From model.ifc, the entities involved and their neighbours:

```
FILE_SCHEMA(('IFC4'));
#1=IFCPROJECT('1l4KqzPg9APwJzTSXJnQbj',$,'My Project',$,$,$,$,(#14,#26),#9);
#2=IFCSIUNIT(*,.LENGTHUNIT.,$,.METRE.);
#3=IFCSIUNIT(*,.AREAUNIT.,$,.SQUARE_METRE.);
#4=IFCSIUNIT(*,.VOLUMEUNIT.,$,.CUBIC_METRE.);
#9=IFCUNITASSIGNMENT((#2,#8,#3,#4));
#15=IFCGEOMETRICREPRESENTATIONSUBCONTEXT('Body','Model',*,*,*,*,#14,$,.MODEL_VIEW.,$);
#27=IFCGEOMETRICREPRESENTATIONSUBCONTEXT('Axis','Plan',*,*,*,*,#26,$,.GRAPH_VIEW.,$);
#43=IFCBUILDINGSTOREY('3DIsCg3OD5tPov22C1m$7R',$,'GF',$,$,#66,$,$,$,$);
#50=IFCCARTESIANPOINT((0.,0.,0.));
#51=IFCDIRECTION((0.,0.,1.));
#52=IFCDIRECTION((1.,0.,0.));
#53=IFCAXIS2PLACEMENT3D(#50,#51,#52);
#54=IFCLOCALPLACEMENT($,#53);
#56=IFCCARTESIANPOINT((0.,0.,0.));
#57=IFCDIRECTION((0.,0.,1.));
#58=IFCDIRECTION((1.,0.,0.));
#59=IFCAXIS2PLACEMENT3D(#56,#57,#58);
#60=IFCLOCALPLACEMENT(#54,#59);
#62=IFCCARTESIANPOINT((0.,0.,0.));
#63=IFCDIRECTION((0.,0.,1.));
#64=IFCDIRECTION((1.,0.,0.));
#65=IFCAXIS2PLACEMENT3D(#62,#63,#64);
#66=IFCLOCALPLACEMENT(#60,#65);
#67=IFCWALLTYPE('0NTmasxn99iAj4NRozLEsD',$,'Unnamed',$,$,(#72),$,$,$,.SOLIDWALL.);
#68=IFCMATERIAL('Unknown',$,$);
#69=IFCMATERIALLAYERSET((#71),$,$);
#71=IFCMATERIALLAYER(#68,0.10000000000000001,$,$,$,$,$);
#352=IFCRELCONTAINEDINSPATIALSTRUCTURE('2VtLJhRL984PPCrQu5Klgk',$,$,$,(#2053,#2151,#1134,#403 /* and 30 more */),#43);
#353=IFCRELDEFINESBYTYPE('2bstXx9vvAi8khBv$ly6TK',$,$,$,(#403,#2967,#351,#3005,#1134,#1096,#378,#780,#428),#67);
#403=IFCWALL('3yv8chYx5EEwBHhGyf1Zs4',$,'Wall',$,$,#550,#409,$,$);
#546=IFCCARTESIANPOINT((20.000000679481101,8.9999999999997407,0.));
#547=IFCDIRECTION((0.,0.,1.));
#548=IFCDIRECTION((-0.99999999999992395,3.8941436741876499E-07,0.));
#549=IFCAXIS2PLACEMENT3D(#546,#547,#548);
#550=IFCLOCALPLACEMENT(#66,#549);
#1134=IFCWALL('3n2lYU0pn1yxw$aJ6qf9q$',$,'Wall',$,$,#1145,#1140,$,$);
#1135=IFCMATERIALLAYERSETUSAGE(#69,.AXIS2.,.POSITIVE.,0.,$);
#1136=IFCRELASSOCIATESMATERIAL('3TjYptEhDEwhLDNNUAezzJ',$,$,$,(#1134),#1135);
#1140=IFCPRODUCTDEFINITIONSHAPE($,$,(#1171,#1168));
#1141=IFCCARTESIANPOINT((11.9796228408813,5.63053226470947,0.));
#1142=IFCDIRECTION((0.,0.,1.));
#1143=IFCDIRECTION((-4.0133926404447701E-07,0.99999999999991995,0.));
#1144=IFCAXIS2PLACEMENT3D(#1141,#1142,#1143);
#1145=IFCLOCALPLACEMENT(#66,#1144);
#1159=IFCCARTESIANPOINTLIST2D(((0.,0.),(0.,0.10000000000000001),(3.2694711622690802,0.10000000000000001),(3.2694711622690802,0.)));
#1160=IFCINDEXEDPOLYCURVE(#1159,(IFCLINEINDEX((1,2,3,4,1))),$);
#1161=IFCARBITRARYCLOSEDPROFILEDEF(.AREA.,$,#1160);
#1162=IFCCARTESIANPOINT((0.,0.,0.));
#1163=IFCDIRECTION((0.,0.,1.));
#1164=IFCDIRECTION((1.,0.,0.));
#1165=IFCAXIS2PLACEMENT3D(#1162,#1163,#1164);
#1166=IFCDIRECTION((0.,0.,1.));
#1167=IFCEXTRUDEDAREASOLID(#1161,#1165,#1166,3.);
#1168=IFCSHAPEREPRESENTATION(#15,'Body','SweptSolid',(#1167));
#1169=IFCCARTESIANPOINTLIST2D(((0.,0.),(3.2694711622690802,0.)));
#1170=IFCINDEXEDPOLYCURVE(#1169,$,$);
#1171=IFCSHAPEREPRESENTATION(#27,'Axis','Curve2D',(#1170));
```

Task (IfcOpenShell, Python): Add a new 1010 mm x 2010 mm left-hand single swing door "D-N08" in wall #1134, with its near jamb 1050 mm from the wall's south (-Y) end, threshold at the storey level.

```python
import numpy as np
import ifcopenshell
import ifcopenshell.api.feature
import ifcopenshell.api.geometry
import ifcopenshell.api.root
import ifcopenshell.api.spatial
import ifcopenshell.geom
import ifcopenshell.util.element
import ifcopenshell.util.placement
import ifcopenshell.util.representation
import ifcopenshell.util.shape
import ifcopenshell.util.unit

model = ifcopenshell.open("model.ifc")
unit_scale = ifcopenshell.util.unit.calculate_unit_scale(model)
settings = ifcopenshell.geom.settings()


def volume(element):
    """Net volume in cubic metres, openings subtracted."""
    shape = ifcopenshell.geom.create_shape(settings, element)
    return ifcopenshell.util.shape.get_volume(shape.geometry)


wall = model.by_id(1134)
storey = ifcopenshell.util.element.get_container(wall, ifc_class="IfcBuildingStorey")
context = ifcopenshell.util.representation.get_context(model, "Model", "Body", "MODEL_VIEW")
before = volume(wall)

width, height, from_end, sill = 1.01, 2.01, 1.05, 0.0  # metres

# The wall runs along its own X axis, and the end named is its -X end.
wall_shape = ifcopenshell.geom.create_shape(settings, wall)
x, y, z = ifcopenshell.util.shape.get_vertices(wall_shape.geometry).T
start = x.min() + from_end
face, thickness = float(y.min()), float(y.max() - y.min())
wall_matrix = ifcopenshell.util.placement.get_local_placement(wall.ObjectPlacement)
level = ifcopenshell.util.placement.get_local_placement(storey.ObjectPlacement)[2, 3]


def in_wall(x, y):
    """Placement at x, y metres in the wall's axes, at sill height."""
    matrix = wall_matrix.copy()
    matrix[:, 3] = wall_matrix @ np.array([x / unit_scale, y / unit_scale, 0.0, 1.0])
    matrix[2, 3] = level + sill / unit_scale
    return matrix


# Opening: a box that overshoots both wall faces by 50 mm.
opening = ifcopenshell.api.root.create_entity(model, ifc_class="IfcOpeningElement", predefined_type="OPENING")
box = ifcopenshell.api.geometry.add_wall_representation(
    model, context=context, length=width, height=height, thickness=thickness + 0.1
)
ifcopenshell.api.geometry.assign_representation(model, product=opening, representation=box)
ifcopenshell.api.geometry.edit_object_placement(model, product=opening, matrix=in_wall(start, face - 0.05), is_si=False)
ifcopenshell.api.feature.add_feature(model, feature=opening, element=wall)

door = ifcopenshell.api.root.create_entity(model, ifc_class="IfcDoor", name="D-N08", predefined_type="DOOR")
door.OverallWidth, door.OverallHeight = width / unit_scale, height / unit_scale
door.OperationType = "SINGLE_SWING_LEFT"
body = ifcopenshell.api.geometry.add_door_representation(
    model,
    context=context,
    overall_width=door.OverallWidth,
    overall_height=door.OverallHeight,
    operation_type="SINGLE_SWING_LEFT",
    lining_properties={"LiningDepth": thickness / unit_scale, "ThresholdDepth": thickness / unit_scale},
)
ifcopenshell.api.geometry.assign_representation(model, product=door, representation=body)
ifcopenshell.api.spatial.assign_container(model, products=[door], relating_structure=storey)
ifcopenshell.api.feature.add_filling(model, opening=opening, element=door)

# The lining spans the wall, so the door starts at the wall face.
ifcopenshell.api.geometry.edit_object_placement(model, product=door, matrix=in_wall(start, face), is_si=False)

after = volume(wall)

print(f"wall volume {before:.3f} -> {after:.3f} m3")

model.write("model_updated.ifc")
```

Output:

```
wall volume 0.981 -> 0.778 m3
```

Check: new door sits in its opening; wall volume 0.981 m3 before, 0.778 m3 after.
